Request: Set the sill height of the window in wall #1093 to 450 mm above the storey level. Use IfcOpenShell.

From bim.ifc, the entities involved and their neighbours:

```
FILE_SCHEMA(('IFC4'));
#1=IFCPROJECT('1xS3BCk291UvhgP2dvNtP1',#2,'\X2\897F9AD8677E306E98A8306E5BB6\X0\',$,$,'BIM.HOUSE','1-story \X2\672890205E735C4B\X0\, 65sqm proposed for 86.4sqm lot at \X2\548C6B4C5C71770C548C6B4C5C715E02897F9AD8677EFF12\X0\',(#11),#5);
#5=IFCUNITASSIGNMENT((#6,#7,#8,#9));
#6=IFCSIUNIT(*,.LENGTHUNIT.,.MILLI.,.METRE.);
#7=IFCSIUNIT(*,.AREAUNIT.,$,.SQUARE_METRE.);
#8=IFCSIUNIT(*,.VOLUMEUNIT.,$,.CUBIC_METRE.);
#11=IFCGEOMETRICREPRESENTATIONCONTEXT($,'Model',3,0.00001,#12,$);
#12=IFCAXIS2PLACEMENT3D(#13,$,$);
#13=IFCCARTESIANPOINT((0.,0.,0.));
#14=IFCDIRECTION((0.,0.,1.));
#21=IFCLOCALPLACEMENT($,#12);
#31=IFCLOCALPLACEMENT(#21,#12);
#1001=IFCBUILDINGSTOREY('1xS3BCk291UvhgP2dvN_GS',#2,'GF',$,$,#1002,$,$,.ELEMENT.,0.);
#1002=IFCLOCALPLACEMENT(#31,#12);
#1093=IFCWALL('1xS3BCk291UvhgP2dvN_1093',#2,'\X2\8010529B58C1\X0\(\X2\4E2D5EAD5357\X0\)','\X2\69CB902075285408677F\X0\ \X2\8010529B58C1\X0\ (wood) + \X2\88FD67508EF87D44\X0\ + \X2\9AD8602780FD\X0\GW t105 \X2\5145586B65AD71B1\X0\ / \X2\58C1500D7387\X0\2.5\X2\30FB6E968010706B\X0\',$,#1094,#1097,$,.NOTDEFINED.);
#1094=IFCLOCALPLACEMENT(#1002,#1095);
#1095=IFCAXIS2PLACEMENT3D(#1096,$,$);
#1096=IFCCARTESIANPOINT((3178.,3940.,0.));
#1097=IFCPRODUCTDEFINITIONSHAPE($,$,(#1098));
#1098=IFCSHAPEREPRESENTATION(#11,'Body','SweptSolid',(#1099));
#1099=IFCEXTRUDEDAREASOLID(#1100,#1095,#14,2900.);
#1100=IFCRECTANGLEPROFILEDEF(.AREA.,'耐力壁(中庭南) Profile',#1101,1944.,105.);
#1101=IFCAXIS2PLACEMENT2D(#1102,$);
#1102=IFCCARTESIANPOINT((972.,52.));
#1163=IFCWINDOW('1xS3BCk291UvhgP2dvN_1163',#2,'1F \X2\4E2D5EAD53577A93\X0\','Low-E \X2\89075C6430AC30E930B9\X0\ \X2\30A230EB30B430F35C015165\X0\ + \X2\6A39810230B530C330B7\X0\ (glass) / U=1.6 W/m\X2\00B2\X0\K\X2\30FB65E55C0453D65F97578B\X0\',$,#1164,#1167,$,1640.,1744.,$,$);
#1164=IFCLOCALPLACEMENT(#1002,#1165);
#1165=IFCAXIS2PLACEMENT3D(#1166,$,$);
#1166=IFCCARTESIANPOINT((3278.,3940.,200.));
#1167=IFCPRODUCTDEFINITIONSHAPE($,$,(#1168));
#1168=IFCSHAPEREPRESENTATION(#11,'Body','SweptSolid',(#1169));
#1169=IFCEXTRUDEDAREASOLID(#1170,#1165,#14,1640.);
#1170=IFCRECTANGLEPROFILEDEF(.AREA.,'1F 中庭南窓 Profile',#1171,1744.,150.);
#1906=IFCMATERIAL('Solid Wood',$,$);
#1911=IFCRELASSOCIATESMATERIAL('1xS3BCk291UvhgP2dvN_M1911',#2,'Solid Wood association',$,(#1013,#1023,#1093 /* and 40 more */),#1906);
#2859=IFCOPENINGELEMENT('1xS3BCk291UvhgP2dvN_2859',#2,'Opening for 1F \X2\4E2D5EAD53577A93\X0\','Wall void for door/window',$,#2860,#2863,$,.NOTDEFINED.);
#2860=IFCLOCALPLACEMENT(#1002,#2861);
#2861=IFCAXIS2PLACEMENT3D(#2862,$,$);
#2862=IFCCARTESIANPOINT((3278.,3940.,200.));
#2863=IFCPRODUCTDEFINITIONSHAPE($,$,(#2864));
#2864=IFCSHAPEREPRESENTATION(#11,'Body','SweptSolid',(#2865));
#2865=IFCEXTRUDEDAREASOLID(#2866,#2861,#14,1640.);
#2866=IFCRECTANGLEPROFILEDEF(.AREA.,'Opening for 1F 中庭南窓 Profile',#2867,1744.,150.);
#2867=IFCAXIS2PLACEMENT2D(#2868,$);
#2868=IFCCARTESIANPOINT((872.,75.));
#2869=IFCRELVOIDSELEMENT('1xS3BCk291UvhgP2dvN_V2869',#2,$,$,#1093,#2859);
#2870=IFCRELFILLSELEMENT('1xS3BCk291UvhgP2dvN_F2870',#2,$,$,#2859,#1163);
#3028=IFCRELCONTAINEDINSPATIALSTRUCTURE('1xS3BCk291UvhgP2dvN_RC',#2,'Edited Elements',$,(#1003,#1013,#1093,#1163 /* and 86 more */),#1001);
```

```python
import numpy as np
import ifcopenshell
import ifcopenshell.api.geometry
import ifcopenshell.geom
import ifcopenshell.util.element
import ifcopenshell.util.placement
import ifcopenshell.util.shape
import ifcopenshell.util.unit

model = ifcopenshell.open("bim.ifc")
unit_scale = ifcopenshell.util.unit.calculate_unit_scale(model)

window = model.by_guid("1xS3BCk291UvhgP2dvN_1163")
opening = window.FillsVoids[0].RelatingOpeningElement
storey = ifcopenshell.util.element.get_container(window, ifc_class="IfcBuildingStorey")
level = ifcopenshell.util.placement.get_local_placement(storey.ObjectPlacement)[2, 3]

# The opening's origin need not be at the sill, so measure its lowest point.
shape = ifcopenshell.geom.create_shape(ifcopenshell.geom.settings(), opening)
bottom = ifcopenshell.util.shape.get_shape_bottom_elevation(shape, shape.geometry) / unit_scale
dz = level + 0.45 / unit_scale - bottom

shift = np.array([0.0, 0.0, dz])
# The window is not placed relative to its opening, so move both.
for product in (opening, window):
    matrix = ifcopenshell.util.placement.get_local_placement(product.ObjectPlacement)
    matrix[:3, 3] += shift
    ifcopenshell.api.geometry.edit_object_placement(model, product=product, matrix=matrix, is_si=False)

print(f"moved by {dz * unit_scale:+.3f} m")

model.write("bim-out.ifc")
```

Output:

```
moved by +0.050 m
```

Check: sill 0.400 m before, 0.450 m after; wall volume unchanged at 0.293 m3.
